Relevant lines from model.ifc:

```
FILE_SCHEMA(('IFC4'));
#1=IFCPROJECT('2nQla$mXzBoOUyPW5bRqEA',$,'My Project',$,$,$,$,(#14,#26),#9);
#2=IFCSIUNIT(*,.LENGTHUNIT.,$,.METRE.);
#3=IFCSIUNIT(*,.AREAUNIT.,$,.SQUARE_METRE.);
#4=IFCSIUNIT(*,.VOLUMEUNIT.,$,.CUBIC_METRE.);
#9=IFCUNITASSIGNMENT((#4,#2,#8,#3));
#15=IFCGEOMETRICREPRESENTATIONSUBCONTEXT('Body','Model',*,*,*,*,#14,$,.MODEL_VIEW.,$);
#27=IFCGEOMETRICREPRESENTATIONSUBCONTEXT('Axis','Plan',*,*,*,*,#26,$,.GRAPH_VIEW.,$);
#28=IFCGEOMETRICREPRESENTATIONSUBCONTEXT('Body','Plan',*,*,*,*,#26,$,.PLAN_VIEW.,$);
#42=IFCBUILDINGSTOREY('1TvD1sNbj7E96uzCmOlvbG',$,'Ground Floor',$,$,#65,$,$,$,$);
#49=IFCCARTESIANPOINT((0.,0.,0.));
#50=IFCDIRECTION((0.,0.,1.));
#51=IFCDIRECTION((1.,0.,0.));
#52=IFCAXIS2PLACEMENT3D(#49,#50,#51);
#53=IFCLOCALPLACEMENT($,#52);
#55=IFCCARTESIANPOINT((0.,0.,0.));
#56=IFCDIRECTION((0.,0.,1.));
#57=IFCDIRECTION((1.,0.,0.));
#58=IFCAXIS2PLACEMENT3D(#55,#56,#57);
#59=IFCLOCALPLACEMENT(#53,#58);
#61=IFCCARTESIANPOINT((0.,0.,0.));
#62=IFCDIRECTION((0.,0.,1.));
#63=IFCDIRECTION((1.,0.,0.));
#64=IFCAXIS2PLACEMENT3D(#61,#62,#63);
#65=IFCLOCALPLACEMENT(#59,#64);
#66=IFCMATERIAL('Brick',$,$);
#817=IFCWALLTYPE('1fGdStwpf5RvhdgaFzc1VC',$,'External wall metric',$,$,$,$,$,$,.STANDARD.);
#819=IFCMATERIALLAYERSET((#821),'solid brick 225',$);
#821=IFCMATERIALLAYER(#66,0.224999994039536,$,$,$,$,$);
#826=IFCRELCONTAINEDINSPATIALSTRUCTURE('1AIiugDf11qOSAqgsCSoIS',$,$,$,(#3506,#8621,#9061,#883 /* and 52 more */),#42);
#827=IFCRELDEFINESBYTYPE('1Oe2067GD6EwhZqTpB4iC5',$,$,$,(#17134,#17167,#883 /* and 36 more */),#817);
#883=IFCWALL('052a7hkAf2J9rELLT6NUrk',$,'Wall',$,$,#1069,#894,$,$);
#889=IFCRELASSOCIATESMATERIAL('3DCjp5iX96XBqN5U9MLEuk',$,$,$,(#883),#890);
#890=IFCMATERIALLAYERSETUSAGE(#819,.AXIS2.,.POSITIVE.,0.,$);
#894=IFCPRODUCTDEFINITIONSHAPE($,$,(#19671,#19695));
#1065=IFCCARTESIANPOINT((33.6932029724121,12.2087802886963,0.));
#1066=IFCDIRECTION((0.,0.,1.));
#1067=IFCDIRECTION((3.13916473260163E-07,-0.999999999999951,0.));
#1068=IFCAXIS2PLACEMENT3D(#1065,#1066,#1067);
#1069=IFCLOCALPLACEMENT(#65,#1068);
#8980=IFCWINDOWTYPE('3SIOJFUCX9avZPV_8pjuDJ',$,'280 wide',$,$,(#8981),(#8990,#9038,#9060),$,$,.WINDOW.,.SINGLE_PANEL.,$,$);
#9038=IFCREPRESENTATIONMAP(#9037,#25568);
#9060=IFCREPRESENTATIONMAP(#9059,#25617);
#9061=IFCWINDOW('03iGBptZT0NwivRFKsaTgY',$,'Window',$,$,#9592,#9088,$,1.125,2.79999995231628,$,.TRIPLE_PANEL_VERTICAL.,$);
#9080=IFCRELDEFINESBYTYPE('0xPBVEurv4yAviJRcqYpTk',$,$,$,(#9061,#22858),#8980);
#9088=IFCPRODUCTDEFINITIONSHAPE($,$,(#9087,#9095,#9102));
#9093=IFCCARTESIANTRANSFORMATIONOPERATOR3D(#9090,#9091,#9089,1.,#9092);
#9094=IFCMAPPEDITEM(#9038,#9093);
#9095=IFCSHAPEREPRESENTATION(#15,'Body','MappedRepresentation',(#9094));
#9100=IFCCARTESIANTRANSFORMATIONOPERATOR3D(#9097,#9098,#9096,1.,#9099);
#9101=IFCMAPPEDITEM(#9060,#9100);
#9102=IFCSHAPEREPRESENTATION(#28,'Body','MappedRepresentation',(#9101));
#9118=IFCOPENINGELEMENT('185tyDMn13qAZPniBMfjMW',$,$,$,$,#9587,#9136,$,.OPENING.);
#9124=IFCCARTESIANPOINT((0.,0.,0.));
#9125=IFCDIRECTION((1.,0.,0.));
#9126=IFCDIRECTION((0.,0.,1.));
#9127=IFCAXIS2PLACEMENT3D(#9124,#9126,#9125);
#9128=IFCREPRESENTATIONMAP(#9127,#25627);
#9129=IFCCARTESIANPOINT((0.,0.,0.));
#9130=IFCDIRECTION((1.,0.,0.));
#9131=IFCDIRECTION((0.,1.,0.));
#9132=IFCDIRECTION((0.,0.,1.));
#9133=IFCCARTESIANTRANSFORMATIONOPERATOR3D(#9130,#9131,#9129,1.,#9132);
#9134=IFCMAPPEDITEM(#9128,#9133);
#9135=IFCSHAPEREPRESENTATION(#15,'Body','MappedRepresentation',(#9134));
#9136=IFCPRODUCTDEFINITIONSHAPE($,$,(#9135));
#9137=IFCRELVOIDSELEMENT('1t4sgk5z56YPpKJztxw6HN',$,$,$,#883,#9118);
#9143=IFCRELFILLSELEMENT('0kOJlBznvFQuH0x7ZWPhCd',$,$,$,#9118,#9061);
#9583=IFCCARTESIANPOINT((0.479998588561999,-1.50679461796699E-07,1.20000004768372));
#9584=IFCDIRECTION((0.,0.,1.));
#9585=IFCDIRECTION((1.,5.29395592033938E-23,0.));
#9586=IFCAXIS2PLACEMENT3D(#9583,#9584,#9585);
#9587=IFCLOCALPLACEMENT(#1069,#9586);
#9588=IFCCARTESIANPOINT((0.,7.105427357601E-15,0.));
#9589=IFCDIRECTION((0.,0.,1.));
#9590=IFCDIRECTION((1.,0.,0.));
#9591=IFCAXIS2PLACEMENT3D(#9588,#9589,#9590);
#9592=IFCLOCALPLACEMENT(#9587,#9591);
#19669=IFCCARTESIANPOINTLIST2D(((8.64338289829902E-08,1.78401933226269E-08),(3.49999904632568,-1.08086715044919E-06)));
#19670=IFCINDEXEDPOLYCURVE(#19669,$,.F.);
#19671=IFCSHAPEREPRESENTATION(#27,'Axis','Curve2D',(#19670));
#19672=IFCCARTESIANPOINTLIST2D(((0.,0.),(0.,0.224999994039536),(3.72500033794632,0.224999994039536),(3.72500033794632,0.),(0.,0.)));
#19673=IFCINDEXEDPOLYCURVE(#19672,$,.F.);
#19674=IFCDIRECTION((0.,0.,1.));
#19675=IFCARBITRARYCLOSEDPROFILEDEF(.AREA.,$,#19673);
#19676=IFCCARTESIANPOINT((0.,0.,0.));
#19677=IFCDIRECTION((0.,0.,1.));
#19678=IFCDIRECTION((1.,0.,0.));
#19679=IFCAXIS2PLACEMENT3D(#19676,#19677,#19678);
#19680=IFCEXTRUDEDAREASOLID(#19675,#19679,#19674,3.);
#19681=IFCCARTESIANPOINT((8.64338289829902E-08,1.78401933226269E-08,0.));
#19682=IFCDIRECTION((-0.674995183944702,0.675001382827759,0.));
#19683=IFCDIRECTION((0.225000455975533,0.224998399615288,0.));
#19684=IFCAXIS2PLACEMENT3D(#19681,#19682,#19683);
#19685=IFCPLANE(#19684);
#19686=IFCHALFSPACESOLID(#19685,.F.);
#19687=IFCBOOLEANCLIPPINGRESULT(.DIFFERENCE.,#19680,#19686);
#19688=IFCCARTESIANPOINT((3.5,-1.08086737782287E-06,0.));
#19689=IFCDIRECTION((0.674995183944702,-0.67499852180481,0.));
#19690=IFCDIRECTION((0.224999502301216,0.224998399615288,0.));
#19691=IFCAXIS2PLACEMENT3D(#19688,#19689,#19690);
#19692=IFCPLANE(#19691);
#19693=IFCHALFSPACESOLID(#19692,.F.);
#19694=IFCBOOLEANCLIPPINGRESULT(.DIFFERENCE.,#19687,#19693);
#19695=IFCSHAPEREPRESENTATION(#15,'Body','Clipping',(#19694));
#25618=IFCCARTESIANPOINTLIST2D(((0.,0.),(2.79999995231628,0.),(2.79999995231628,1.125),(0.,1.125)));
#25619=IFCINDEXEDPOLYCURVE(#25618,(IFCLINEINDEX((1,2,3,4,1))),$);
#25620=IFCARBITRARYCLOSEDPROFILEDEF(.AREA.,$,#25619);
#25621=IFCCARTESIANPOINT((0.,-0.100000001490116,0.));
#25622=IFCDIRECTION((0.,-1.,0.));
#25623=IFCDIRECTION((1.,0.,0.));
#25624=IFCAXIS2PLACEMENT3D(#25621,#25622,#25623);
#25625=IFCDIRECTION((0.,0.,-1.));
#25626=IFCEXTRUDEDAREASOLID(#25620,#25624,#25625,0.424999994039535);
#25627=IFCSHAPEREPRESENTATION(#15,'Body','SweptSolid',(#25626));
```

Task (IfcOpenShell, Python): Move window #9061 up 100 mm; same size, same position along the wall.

```python
import numpy as np
import ifcopenshell
import ifcopenshell.api.geometry
import ifcopenshell.util.placement
import ifcopenshell.util.unit

model = ifcopenshell.open("model.ifc")
unit_scale = ifcopenshell.util.unit.calculate_unit_scale(model)

window = model.by_guid("03iGBptZT0NwivRFKsaTgY")
opening = window.FillsVoids[0].RelatingOpeningElement
dz = 0.1 / unit_scale

shift = np.array([0.0, 0.0, dz])
# The window is placed relative to its opening, so it follows when the opening moves.
matrix = ifcopenshell.util.placement.get_local_placement(opening.ObjectPlacement)
matrix[:3, 3] += shift
ifcopenshell.api.geometry.edit_object_placement(
    model, product=opening, matrix=matrix, is_si=False, should_transform_children=True
)

print(f"moved by {dz * unit_scale:+.3f} m")

model.write("model_edited.ifc")
```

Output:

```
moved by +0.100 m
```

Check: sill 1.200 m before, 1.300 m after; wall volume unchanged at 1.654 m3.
